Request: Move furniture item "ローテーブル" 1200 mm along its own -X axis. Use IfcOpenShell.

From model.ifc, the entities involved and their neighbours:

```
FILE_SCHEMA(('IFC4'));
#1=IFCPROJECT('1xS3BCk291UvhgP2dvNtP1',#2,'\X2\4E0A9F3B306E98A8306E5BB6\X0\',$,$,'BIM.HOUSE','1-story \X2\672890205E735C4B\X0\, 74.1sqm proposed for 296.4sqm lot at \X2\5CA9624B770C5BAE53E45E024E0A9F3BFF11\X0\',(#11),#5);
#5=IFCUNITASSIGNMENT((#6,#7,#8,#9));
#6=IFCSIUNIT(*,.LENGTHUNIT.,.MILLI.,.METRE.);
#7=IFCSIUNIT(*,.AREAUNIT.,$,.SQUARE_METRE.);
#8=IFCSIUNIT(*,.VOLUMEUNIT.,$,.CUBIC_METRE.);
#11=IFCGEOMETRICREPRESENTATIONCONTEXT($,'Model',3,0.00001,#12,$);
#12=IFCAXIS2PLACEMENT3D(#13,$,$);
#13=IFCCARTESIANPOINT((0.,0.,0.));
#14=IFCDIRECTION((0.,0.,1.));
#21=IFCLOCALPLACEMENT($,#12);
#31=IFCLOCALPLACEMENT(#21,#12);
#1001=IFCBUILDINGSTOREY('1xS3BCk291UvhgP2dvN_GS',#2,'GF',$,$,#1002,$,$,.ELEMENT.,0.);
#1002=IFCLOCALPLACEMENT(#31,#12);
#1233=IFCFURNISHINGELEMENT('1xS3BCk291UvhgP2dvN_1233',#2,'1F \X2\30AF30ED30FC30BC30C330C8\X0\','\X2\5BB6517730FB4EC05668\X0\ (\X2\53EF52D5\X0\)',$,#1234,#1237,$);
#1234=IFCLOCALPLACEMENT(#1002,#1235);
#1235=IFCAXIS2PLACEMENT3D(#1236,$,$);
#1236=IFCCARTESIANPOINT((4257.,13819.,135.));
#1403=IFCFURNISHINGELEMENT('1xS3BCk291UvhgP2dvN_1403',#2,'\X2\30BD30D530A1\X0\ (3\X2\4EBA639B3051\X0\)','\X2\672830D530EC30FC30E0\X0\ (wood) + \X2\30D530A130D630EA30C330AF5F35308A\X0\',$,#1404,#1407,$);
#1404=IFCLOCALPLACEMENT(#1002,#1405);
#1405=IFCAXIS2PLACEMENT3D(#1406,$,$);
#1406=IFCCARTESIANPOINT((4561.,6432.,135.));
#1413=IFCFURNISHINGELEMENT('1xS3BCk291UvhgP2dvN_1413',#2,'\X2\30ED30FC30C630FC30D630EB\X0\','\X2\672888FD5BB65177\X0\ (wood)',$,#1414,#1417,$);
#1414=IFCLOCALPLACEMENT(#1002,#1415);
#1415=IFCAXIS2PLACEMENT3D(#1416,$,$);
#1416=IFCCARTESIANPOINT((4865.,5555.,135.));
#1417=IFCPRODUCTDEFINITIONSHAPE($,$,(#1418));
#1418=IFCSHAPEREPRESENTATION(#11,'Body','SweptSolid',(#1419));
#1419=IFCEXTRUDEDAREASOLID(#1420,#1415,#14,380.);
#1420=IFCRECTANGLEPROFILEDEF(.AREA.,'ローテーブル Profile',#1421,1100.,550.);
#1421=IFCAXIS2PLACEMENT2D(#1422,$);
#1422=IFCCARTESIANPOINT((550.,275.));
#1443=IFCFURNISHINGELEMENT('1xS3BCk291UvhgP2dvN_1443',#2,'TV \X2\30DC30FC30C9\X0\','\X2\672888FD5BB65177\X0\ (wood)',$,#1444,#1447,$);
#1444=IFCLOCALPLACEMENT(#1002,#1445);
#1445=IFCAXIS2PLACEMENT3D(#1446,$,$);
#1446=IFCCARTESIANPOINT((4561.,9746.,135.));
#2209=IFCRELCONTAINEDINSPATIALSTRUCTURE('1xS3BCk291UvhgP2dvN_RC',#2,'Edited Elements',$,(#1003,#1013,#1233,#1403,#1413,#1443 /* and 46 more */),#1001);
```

```python
import ifcopenshell
import ifcopenshell.api.geometry
import ifcopenshell.util.placement
import ifcopenshell.util.unit

model = ifcopenshell.open("model.ifc")
unit_scale = ifcopenshell.util.unit.calculate_unit_scale(model)

item = model.by_id(1413)
matrix = ifcopenshell.util.placement.get_local_placement(item.ObjectPlacement)
matrix[:3, 3] -= matrix[:3, 0] * 1.2 / unit_scale
ifcopenshell.api.geometry.edit_object_placement(model, product=item, matrix=matrix, is_si=False)

print(ifcopenshell.util.placement.get_local_placement(item.ObjectPlacement).round(3) + 0.0)

model.write("model_rev.ifc")
```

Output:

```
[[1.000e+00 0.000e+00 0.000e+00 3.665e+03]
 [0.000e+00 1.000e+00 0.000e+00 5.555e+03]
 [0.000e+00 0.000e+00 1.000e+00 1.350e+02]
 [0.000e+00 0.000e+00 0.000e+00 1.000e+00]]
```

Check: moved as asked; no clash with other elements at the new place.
